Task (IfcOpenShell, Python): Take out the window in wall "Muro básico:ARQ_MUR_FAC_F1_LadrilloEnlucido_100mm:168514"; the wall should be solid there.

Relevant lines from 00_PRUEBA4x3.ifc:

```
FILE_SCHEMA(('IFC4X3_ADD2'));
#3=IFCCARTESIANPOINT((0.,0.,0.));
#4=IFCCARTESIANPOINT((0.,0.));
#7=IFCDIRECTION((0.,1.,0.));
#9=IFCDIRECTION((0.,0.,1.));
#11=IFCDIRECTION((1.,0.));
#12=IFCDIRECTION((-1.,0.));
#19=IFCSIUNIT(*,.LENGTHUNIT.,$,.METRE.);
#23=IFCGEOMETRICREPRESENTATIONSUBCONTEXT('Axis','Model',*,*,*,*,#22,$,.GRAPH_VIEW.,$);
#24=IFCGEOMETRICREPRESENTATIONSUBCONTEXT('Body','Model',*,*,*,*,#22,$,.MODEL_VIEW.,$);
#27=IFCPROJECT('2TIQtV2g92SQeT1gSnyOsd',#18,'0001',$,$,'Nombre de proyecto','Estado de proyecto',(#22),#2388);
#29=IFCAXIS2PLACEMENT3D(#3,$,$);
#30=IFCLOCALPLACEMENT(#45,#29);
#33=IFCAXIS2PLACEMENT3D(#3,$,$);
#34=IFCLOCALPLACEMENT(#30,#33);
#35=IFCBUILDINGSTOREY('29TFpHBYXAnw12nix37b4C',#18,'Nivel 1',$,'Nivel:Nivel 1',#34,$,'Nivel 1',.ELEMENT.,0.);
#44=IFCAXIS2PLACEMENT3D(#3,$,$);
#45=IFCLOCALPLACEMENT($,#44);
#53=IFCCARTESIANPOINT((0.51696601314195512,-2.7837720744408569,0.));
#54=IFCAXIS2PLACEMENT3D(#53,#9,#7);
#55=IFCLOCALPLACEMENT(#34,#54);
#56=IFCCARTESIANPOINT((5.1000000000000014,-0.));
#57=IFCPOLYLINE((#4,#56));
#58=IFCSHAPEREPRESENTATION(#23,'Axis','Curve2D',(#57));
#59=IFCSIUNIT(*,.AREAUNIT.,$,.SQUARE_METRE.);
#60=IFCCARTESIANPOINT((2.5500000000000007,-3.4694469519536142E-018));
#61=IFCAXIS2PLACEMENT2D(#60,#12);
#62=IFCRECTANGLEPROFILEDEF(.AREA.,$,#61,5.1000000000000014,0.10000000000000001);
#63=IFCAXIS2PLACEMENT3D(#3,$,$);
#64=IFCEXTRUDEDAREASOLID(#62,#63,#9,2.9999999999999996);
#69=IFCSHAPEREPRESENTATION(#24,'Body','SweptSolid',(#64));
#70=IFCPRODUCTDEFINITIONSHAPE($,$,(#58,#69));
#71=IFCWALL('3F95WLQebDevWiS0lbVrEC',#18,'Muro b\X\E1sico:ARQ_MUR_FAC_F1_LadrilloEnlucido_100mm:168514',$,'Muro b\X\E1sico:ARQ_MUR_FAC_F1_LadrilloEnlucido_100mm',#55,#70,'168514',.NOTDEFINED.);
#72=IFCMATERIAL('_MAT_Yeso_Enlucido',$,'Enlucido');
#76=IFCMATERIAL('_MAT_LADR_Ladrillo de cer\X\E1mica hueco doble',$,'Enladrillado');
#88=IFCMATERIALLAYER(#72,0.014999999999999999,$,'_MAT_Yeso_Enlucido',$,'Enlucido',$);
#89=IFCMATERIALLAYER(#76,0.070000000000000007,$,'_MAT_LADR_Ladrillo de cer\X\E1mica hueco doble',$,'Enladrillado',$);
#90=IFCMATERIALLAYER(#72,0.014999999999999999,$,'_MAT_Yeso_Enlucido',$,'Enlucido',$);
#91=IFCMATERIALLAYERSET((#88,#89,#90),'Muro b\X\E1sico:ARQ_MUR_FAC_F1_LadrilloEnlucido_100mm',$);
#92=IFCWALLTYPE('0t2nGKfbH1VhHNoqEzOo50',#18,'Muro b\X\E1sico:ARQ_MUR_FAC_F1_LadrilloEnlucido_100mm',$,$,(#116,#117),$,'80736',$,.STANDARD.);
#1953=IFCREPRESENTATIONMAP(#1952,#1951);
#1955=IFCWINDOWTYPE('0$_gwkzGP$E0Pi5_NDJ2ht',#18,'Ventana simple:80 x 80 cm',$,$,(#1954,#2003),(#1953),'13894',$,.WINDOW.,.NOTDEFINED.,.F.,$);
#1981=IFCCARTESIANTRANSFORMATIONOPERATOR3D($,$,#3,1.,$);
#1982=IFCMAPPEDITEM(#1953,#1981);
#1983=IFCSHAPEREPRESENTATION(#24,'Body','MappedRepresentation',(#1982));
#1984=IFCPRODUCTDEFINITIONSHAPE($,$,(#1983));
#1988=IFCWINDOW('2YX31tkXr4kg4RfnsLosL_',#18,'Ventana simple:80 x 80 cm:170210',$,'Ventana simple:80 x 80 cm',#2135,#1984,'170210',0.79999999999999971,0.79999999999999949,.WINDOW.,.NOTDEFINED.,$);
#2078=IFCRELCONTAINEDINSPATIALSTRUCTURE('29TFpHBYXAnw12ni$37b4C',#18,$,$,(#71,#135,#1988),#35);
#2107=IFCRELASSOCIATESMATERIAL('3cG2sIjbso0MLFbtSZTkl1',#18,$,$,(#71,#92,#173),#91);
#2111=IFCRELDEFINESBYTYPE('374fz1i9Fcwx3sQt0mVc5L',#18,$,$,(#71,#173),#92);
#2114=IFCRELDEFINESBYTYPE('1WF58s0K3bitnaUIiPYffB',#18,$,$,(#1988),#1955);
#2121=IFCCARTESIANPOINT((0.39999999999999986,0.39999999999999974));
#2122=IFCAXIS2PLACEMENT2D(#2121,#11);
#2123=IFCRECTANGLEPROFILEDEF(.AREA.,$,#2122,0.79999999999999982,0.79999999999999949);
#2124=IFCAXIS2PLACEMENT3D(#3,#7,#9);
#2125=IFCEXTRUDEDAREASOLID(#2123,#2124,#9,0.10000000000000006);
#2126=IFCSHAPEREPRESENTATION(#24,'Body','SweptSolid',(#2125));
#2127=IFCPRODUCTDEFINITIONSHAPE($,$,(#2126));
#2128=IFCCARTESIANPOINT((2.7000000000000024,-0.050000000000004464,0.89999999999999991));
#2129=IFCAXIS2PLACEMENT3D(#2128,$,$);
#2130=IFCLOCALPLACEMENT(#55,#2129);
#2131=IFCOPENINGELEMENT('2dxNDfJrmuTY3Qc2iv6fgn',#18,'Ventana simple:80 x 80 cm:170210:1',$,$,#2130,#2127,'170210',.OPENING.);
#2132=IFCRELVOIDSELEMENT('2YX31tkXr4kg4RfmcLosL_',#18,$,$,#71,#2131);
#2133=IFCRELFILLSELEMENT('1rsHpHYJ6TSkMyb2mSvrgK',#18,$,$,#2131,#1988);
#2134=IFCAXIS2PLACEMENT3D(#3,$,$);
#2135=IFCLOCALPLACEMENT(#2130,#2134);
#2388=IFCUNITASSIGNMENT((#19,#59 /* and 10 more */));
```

```python
import ifcopenshell
import ifcopenshell.api.feature
import ifcopenshell.api.root
import ifcopenshell.geom
import ifcopenshell.util.shape

model = ifcopenshell.open("00_PRUEBA4x3.ifc")
settings = ifcopenshell.geom.settings()


def volume(element):
    """Net volume in cubic metres, openings subtracted."""
    shape = ifcopenshell.geom.create_shape(settings, element)
    return ifcopenshell.util.shape.get_volume(shape.geometry)


window = model.by_guid("2YX31tkXr4kg4RfnsLosL_")
opening = window.FillsVoids[0].RelatingOpeningElement
wall = opening.VoidsElements[0].RelatingBuildingElement
before = volume(wall)

ifcopenshell.api.root.remove_product(model, product=window)
ifcopenshell.api.feature.remove_feature(model, feature=opening)

after = volume(wall)

print(f"wall volume {before:.3f} -> {after:.3f} m3")

model.write("00_PRUEBA4x3_v2.ifc")
```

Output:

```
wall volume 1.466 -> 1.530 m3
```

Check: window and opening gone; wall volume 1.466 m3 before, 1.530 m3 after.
